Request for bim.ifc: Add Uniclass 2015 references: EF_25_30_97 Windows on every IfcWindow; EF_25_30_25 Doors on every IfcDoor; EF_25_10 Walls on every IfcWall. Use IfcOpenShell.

First a look at what the model holds.

```python
import ifcopenshell

model = ifcopenshell.open("bim.ifc")
print(model.schema)
print("classifications:", [c.Name for c in model.by_type("IfcClassification")])
for ifc_class in ("IfcDoor", "IfcRoof", "IfcStair", "IfcWall", "IfcWindow"):
    print(ifc_class, len(model.by_type(ifc_class)))
```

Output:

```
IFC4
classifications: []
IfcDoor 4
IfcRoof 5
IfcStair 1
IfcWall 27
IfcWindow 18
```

```python
import ifcopenshell
import ifcopenshell.api.classification

model = ifcopenshell.open("bim.ifc")

system = ifcopenshell.api.classification.add_classification(model, classification="Uniclass 2015")

codes = {
    "IfcWindow": ("EF_25_30_97", "Windows"),
    "IfcDoor": ("EF_25_30_25", "Doors"),
    "IfcWall": ("EF_25_10", "Walls"),
}
for ifc_class, (code, name) in codes.items():
    products = model.by_type(ifc_class)
    ifcopenshell.api.classification.add_reference(
        model, products=products, classification=system, identification=code, name=name
    )
    print(code, len(products))

model.write("bim-out.ifc")
```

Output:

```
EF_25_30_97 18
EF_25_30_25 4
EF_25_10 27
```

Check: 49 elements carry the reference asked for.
